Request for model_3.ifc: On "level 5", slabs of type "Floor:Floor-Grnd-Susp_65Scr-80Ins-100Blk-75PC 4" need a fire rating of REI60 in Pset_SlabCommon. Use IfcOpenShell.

First a look at what the model holds.

```python
import ifcopenshell
import ifcopenshell.util.element

model = ifcopenshell.open("model_3.ifc")
print(model.schema)
storey = next(s for s in model.by_type("IfcBuildingStorey") if s.Name == "level 5")
slabs = [e for e in ifcopenshell.util.element.get_decomposition(storey) if e.is_a("IfcSlab")]
seen = {}
for e in slabs:
    element_type = ifcopenshell.util.element.get_type(e)
    key = (element_type.Name if element_type != e and element_type else None, ifcopenshell.util.element.get_pset(e, "Pset_SlabCommon", "FireRating"))
    seen[key] = seen.get(key, 0) + 1
for (name, value), count in sorted(seen.items(), key=str):
    print(count, "x", name, "|", value)
```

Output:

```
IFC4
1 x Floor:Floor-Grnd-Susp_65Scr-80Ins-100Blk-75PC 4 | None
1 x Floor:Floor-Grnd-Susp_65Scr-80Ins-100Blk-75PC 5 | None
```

```python
import ifcopenshell
import ifcopenshell.api.pset
import ifcopenshell.util.element

model = ifcopenshell.open("model_3.ifc")

storey = next(s for s in model.by_type("IfcBuildingStorey") if s.Name == "level 5")
slabs = [e for e in ifcopenshell.util.element.get_decomposition(storey) if e.is_a("IfcSlab")]

count = 0
for e in slabs:
    element_type = ifcopenshell.util.element.get_type(e)
    if element_type in (None, e) or element_type.Name != "Floor:Floor-Grnd-Susp_65Scr-80Ins-100Blk-75PC 4":
        continue
    # add_pset returns the element's existing set when there is one.
    pset = ifcopenshell.api.pset.add_pset(model, product=e, name="Pset_SlabCommon")
    ifcopenshell.api.pset.edit_pset(model, pset=pset, properties={"FireRating": "REI60"})
    count += 1

print(count, "slabs updated")

model.write("model_3-out.ifc")
```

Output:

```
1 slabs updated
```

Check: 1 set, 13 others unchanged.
